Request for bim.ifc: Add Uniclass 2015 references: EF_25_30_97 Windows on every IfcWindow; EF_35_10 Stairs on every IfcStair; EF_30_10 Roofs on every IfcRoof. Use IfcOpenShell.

First a look at what the model holds.

```python
import ifcopenshell

model = ifcopenshell.open("bim.ifc")
print(model.schema)
print("classifications:", [c.Name for c in model.by_type("IfcClassification")])
for ifc_class in ("IfcDoor", "IfcRoof", "IfcStair", "IfcWall", "IfcWindow"):
    print(ifc_class, len(model.by_type(ifc_class)))
```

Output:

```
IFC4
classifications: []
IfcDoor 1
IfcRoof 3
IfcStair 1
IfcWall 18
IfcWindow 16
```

```python
import ifcopenshell
import ifcopenshell.api.classification

model = ifcopenshell.open("bim.ifc")

system = ifcopenshell.api.classification.add_classification(model, classification="Uniclass 2015")

codes = {
    "IfcWindow": ("EF_25_30_97", "Windows"),
    "IfcStair": ("EF_35_10", "Stairs"),
    "IfcRoof": ("EF_30_10", "Roofs"),
}
for ifc_class, (code, name) in codes.items():
    products = model.by_type(ifc_class)
    ifcopenshell.api.classification.add_reference(
        model, products=products, classification=system, identification=code, name=name
    )
    print(code, len(products))

model.write("bim_rev.ifc")
```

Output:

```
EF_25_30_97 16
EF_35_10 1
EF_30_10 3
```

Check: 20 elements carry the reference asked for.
